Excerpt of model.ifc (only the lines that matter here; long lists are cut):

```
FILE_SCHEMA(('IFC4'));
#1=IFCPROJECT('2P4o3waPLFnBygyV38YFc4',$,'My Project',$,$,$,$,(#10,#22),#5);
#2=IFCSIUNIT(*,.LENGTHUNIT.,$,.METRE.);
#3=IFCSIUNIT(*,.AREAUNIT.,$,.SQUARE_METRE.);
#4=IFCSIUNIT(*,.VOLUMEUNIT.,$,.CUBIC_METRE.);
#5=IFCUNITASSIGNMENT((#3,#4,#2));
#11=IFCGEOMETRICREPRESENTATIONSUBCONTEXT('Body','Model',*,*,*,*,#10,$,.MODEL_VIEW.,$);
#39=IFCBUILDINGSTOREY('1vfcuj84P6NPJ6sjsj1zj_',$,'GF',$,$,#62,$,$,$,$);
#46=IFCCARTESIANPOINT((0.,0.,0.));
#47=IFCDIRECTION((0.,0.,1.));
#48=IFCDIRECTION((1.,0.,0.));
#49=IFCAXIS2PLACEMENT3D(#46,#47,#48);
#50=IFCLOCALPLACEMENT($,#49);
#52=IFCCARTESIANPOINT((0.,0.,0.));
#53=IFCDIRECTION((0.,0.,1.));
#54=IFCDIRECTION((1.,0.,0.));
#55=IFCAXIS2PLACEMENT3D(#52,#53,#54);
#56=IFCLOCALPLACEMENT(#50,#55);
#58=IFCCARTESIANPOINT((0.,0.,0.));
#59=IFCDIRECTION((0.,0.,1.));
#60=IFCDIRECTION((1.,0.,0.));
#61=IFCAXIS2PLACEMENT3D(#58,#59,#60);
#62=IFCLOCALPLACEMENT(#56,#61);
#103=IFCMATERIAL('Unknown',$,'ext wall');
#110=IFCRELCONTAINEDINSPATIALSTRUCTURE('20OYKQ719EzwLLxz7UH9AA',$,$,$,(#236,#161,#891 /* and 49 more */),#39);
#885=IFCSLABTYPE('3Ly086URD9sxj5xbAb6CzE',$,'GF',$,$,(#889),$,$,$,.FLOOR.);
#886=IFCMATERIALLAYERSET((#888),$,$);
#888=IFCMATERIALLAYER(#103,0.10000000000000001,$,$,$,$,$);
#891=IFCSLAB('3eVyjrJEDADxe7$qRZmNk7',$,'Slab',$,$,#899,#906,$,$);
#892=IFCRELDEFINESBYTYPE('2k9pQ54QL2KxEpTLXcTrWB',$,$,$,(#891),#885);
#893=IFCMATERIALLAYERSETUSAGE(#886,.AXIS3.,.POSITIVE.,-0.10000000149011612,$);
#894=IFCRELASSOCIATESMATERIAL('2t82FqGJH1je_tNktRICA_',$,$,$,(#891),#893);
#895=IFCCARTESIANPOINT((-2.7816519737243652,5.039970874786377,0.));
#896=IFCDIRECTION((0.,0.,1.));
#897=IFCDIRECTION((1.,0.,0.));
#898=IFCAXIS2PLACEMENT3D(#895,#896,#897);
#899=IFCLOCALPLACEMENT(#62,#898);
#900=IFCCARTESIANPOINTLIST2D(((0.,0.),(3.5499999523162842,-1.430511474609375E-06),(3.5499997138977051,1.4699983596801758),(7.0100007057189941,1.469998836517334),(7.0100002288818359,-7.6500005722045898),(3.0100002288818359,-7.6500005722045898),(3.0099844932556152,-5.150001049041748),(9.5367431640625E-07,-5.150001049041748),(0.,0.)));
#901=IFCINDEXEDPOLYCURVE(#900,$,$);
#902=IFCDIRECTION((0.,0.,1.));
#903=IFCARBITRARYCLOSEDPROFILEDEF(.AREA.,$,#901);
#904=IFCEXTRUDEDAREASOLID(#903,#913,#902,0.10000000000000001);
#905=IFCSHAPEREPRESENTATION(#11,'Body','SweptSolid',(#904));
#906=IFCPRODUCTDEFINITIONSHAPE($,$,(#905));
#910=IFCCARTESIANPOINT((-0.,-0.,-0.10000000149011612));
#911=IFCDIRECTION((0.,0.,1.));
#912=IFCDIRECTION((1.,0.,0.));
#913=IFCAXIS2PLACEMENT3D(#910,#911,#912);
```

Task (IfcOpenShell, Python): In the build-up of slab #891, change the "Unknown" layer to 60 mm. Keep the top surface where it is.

```python
import ifcopenshell
import ifcopenshell.util.element
import ifcopenshell.util.representation
import ifcopenshell.util.unit

model = ifcopenshell.open("model.ifc")
unit_scale = ifcopenshell.util.unit.calculate_unit_scale(model)

layer_set = model.by_id(886)
layer = next(l for l in layer_set.MaterialLayers if l.Material and l.Material.Name == "Unknown")
change = 0.06 / unit_scale - layer.LayerThickness
layer.LayerThickness += change

# Geometry does not follow the layer set by itself.
slabs = [e for e in ifcopenshell.util.element.get_elements_by_material(model, layer_set) if e.is_a("IfcSlab")]
for slab in sorted(slabs, key=lambda e: e.id()):
    body = ifcopenshell.util.representation.get_representation(slab, "Model", "Body")
    solid = body.Items[0]
    old_depth = solid.Depth
    solid.Depth += change
    # Extruded upwards: lower the start of the extrusion so the top stays.
    x, y, z = solid.Position.Location.Coordinates
    solid.Position.Location = model.createIfcCartesianPoint((x, y, z - change))
    print(slab.id(), f"{old_depth:g} -> {solid.Depth:g}")

# The layers are counted up from the underside, which has moved.
for usage in {ifcopenshell.util.element.get_material(slab) for slab in slabs}:
    usage.OffsetFromReferenceLine -= change

model.write("model_rev.ifc")
```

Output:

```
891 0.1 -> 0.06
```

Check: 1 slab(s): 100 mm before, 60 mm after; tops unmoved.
